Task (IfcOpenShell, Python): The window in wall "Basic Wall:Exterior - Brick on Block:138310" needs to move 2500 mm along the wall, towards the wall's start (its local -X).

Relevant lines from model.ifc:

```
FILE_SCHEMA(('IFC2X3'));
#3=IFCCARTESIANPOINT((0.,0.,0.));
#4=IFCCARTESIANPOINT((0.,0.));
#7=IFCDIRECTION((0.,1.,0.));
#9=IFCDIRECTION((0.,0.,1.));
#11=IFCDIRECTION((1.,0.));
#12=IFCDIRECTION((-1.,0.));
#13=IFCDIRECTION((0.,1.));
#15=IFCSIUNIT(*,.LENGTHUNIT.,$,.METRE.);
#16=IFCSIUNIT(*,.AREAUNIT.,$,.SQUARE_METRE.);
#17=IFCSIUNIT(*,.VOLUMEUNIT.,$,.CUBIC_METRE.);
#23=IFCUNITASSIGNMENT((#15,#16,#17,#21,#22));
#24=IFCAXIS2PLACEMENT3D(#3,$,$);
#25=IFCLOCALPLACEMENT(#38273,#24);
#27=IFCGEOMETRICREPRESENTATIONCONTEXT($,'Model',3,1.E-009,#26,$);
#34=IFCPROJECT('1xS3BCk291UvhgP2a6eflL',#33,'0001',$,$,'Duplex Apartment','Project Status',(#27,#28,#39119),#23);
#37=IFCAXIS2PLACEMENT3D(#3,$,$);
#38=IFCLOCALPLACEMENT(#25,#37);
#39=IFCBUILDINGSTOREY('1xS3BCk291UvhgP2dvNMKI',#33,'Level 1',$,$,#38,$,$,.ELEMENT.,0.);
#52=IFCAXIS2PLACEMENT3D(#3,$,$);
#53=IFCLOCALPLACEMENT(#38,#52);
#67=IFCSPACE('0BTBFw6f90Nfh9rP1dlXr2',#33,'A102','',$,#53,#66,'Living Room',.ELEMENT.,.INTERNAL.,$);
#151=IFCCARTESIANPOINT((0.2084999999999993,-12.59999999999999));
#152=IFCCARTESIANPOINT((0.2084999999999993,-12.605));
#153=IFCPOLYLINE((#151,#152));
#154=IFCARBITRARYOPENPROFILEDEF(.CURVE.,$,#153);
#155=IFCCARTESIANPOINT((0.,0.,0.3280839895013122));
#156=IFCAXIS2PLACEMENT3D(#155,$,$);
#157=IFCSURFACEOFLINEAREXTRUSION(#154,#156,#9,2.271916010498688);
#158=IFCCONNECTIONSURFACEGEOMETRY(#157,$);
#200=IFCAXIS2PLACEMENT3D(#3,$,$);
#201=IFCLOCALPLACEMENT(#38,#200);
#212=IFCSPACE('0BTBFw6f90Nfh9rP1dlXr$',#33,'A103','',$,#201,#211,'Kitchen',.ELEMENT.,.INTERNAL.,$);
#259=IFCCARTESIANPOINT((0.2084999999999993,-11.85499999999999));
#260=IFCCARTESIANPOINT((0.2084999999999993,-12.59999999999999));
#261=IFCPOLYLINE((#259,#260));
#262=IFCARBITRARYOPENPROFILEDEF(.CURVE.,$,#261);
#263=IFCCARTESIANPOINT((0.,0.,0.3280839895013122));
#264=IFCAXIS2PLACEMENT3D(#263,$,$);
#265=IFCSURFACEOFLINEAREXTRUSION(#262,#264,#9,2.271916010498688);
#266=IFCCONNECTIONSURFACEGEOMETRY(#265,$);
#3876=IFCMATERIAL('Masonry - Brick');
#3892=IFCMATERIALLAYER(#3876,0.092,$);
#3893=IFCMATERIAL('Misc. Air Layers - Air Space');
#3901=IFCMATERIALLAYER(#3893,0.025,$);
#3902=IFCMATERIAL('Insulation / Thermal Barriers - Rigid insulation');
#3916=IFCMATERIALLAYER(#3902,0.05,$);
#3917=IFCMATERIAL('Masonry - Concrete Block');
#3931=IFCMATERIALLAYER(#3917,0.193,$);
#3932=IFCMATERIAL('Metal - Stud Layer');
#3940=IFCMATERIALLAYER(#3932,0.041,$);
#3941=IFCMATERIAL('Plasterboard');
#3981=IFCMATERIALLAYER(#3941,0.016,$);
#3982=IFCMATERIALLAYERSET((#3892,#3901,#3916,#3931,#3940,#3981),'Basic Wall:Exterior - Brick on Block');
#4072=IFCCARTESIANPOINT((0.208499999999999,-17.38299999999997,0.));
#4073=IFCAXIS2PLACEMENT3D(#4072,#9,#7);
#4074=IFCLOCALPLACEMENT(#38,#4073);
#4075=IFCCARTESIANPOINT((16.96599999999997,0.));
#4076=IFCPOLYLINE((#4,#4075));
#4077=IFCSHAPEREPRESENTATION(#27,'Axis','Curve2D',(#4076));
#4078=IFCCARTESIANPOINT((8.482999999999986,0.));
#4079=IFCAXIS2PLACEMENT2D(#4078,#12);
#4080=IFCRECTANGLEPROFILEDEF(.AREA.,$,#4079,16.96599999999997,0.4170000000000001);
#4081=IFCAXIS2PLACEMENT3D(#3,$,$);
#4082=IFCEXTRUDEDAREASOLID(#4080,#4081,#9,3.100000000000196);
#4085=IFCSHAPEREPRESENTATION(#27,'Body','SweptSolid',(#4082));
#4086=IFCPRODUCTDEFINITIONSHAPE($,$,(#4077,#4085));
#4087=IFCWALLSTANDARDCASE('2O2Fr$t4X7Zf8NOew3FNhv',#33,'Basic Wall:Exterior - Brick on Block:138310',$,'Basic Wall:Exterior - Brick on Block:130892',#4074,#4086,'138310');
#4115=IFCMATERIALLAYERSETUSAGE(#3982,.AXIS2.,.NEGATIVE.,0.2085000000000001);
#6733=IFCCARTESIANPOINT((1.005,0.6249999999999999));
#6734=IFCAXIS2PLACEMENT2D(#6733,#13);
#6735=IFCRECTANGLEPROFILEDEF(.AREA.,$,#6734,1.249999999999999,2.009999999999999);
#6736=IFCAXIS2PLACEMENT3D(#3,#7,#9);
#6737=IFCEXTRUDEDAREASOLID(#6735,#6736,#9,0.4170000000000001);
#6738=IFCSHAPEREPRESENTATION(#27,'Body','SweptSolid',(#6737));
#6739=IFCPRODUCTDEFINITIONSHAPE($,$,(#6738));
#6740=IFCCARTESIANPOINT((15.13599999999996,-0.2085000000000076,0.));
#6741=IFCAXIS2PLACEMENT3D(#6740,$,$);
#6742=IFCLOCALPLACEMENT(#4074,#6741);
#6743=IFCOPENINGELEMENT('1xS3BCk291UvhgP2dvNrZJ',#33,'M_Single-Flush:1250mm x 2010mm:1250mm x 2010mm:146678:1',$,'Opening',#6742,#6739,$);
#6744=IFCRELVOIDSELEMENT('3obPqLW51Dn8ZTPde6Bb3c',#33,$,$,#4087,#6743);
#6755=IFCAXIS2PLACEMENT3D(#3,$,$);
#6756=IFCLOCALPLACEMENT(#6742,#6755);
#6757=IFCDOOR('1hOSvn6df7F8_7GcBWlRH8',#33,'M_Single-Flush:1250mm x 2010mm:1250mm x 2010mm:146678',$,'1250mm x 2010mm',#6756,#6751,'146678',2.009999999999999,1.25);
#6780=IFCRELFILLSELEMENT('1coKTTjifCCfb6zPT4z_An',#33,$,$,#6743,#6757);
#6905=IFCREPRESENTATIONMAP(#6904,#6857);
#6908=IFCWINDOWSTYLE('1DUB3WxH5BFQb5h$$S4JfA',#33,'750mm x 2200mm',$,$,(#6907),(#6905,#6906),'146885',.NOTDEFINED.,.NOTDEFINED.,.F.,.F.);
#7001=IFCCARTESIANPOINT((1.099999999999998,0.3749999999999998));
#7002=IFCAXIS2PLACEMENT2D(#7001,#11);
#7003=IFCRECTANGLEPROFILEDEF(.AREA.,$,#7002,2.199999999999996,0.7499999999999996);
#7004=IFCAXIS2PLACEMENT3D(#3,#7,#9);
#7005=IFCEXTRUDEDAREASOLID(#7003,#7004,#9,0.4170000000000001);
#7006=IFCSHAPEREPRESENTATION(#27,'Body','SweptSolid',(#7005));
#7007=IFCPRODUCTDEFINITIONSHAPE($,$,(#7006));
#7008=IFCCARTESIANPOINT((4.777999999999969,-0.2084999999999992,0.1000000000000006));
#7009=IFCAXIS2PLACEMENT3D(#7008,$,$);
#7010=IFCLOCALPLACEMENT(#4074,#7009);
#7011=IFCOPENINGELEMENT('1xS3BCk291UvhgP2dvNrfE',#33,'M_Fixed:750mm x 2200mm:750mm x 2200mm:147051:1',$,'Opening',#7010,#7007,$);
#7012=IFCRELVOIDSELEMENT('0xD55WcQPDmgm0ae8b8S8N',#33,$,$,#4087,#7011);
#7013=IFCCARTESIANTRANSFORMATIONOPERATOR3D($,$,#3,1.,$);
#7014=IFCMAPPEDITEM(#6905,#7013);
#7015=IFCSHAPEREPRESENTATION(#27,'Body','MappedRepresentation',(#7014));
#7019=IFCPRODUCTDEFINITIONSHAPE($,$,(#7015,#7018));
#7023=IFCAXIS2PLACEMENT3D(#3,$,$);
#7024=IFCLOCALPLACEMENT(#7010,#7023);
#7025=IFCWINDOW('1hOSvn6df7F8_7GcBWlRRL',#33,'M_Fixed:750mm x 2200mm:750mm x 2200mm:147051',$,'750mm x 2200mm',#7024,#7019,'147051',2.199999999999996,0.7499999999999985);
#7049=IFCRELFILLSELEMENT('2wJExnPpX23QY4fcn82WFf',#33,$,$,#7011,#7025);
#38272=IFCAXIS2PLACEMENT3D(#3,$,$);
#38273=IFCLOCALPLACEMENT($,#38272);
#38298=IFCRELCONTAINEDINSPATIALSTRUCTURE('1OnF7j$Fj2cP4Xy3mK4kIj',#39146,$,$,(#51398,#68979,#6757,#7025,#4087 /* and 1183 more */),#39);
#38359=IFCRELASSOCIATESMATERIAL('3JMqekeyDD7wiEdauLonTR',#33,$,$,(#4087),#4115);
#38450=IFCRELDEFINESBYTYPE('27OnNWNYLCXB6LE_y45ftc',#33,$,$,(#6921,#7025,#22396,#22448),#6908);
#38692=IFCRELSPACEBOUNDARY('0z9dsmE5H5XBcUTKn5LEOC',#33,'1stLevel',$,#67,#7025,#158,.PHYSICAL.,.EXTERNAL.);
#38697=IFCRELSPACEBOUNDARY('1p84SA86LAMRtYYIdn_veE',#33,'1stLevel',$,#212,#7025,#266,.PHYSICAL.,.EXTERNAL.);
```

```python
import numpy as np
import ifcopenshell
import ifcopenshell.api.geometry
import ifcopenshell.util.placement
import ifcopenshell.util.unit

model = ifcopenshell.open("model.ifc")
unit_scale = ifcopenshell.util.unit.calculate_unit_scale(model)

window = model.by_guid("1hOSvn6df7F8_7GcBWlRRL")
opening = window.FillsVoids[0].RelatingOpeningElement
wall = opening.VoidsElements[0].RelatingBuildingElement

wall_matrix = ifcopenshell.util.placement.get_local_placement(wall.ObjectPlacement)
shift = wall_matrix[:3, 0] * -2.5 / unit_scale
before = ifcopenshell.util.placement.get_local_placement(window.ObjectPlacement)[:3, 3].copy()

# The window is placed relative to its opening, so it follows when the opening moves.
matrix = ifcopenshell.util.placement.get_local_placement(opening.ObjectPlacement)
matrix[:3, 3] += shift
ifcopenshell.api.geometry.edit_object_placement(
    model, product=opening, matrix=matrix, is_si=False, should_transform_children=True
)

# Space boundary surfaces are stored in each space's coordinates; move them too.
for rel in window.ProvidesBoundaries:
    if not rel.ConnectionGeometry:
        continue
    surface = rel.ConnectionGeometry.SurfaceOnRelatingElement
    space_matrix = ifcopenshell.util.placement.get_local_placement(rel.RelatingSpace.ObjectPlacement)
    point = np.array(surface.Position.Location.Coordinates) + space_matrix[:3, :3].T @ shift
    surface.Position = model.createIfcAxis2Placement3D(
        model.createIfcCartesianPoint(point.tolist()), surface.Position.Axis, surface.Position.RefDirection
    )

after = ifcopenshell.util.placement.get_local_placement(window.ObjectPlacement)[:3, 3]
print("window moved by", (after - before).round(3) + 0.0)

model.write("model_edited.ifc")
```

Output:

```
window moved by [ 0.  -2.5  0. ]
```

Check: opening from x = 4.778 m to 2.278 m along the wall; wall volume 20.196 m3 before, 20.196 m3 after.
